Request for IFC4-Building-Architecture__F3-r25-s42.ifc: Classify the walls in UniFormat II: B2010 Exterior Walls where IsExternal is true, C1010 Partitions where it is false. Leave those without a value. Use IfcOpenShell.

First a look at what the model holds.

```python
import ifcopenshell
import ifcopenshell.util.element

model = ifcopenshell.open("IFC4-Building-Architecture__F3-r25-s42.ifc")
print(model.schema)
print("classifications:", [c.Name for c in model.by_type("IfcClassification")])
values = [ifcopenshell.util.element.get_pset(e, "Pset_WallCommon", "IsExternal") for e in model.by_type("IfcWall")]
for value in (True, False, None):
    print("IsExternal", value, values.count(value))
```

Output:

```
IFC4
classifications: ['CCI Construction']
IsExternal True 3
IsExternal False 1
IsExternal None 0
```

```python
import ifcopenshell
import ifcopenshell.api.classification
import ifcopenshell.util.element

model = ifcopenshell.open("IFC4-Building-Architecture__F3-r25-s42.ifc")

system = ifcopenshell.api.classification.add_classification(model, classification="UniFormat II")

walls = model.by_type("IfcWall")
external = {e: ifcopenshell.util.element.get_pset(e, "Pset_WallCommon", "IsExternal") for e in walls}
for flag, code, name in ((True, "B2010", "Exterior Walls"), (False, "C1010", "Partitions")):
    products = [e for e in walls if external[e] is flag]
    ifcopenshell.api.classification.add_reference(
        model, products=products, classification=system, identification=code, name=name
    )
    print(code, len(products))

model.write("IFC4-Building-Architecture__F3-r25-s42_updated.ifc")
```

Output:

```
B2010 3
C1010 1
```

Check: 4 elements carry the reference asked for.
